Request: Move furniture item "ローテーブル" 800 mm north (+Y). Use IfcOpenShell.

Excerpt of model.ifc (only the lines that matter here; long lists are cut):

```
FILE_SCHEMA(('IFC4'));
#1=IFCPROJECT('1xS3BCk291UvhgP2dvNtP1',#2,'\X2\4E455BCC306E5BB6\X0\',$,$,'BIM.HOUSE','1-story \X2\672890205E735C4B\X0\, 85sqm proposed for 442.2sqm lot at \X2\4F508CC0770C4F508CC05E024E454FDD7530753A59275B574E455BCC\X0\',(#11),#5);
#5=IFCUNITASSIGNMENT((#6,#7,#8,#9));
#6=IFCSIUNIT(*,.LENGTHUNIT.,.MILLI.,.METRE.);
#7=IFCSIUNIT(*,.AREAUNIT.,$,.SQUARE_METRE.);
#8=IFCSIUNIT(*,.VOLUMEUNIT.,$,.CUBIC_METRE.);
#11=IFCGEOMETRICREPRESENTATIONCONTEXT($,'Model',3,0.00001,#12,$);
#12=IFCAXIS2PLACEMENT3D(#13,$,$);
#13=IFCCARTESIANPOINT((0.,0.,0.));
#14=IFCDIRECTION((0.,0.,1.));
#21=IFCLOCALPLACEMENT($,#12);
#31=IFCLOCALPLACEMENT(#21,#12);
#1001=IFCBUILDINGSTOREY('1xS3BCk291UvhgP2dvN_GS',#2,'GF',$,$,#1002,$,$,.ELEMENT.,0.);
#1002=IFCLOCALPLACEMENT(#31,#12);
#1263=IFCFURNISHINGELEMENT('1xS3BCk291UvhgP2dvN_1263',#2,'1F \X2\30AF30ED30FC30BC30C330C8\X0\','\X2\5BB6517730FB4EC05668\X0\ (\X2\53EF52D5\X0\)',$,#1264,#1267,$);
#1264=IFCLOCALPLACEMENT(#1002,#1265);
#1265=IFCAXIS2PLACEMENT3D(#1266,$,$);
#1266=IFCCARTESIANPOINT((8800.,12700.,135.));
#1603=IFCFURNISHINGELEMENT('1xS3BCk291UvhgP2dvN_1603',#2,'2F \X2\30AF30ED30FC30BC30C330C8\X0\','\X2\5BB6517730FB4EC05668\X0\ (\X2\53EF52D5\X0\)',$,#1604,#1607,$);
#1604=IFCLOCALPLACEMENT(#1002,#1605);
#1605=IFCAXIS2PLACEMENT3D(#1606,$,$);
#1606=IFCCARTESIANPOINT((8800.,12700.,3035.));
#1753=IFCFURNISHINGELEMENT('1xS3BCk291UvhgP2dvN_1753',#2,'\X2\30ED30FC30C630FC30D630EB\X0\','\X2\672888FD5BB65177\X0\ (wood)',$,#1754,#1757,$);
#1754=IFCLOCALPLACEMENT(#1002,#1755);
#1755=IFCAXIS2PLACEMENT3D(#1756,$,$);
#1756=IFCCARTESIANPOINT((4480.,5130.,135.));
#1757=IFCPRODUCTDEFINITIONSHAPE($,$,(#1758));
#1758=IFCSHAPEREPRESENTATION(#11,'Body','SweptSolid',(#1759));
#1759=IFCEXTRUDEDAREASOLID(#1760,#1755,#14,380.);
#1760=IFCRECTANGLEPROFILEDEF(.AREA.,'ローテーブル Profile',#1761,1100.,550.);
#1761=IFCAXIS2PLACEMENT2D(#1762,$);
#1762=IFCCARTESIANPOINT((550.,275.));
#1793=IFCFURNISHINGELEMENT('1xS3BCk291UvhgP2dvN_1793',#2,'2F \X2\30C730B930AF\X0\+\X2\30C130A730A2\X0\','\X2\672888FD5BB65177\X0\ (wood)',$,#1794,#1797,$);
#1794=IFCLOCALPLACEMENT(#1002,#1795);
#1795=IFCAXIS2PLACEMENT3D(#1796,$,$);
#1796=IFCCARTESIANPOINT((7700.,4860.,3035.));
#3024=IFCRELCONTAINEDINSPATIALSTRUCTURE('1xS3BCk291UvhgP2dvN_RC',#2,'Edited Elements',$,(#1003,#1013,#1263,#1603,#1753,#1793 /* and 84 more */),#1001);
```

```python
import ifcopenshell
import ifcopenshell.api.geometry
import ifcopenshell.util.placement
import ifcopenshell.util.unit

model = ifcopenshell.open("model.ifc")
unit_scale = ifcopenshell.util.unit.calculate_unit_scale(model)

item = model.by_guid("1xS3BCk291UvhgP2dvN_1753")
matrix = ifcopenshell.util.placement.get_local_placement(item.ObjectPlacement)
matrix[1, 3] += 0.8 / unit_scale
ifcopenshell.api.geometry.edit_object_placement(model, product=item, matrix=matrix, is_si=False)

print(ifcopenshell.util.placement.get_local_placement(item.ObjectPlacement).round(3) + 0.0)

model.write("model_v2.ifc")
```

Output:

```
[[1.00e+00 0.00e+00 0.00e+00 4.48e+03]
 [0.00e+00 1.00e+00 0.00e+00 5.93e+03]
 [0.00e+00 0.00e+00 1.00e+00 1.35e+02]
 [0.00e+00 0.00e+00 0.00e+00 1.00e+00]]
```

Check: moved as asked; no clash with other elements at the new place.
